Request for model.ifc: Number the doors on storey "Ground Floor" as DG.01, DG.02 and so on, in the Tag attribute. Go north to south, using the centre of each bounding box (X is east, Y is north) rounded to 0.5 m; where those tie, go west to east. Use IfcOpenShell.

First a look at what the model holds.

```python
import ifcopenshell
import ifcopenshell.util.element
import ifcopenshell.util.placement

model = ifcopenshell.open("model.ifc")
print(model.schema)
storey = next(s for s in model.by_type("IfcBuildingStorey") if s.Name == "Ground Floor")
doors = [e for e in ifcopenshell.util.element.get_decomposition(storey) if e.is_a("IfcDoor")]
for e in sorted(doors, key=lambda e: e.id()):
    origin = ifcopenshell.util.placement.get_local_placement(e.ObjectPlacement)[:3, 3]
    print(e.id(), e.Tag, e.Name, origin.round(2) + 0.0, sep=" | ")
```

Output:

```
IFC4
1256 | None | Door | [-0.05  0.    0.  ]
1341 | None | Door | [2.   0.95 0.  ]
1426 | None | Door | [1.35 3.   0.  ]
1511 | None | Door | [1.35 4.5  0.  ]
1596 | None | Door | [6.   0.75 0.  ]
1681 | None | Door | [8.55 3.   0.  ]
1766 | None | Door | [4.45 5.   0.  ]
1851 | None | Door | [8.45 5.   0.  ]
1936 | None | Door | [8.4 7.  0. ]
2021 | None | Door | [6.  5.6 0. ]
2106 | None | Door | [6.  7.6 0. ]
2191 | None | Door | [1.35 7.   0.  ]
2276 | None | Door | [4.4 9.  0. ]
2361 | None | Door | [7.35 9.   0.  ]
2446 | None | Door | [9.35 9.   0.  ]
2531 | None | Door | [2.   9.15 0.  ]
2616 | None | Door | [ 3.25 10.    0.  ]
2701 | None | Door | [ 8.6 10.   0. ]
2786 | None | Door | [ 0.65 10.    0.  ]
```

```python
import ifcopenshell
import ifcopenshell.geom
import ifcopenshell.util.element
import ifcopenshell.util.shape

model = ifcopenshell.open("model.ifc")
settings = ifcopenshell.geom.settings()
settings.set("use-world-coords", True)


def centre(element):
    shape = ifcopenshell.geom.create_shape(settings, element)
    return ifcopenshell.util.shape.get_bbox_centroid(shape.geometry)


storey = next(s for s in model.by_type("IfcBuildingStorey") if s.Name == "Ground Floor")
doors = [e for e in ifcopenshell.util.element.get_decomposition(storey) if e.is_a("IfcDoor")]

# Insertion points can sit at a corner or the storey origin, so sort by the geometry (in metres).
centres = {e: centre(e) for e in doors}
doors.sort(key=lambda e: (-round(centres[e][1] / 0.5), centres[e][0]))

for i, e in enumerate(doors, start=1):
    number = f"DG.{i:02d}"
    e.Tag = number
    print(e.id(), number)

model.write("model-out.ifc")
```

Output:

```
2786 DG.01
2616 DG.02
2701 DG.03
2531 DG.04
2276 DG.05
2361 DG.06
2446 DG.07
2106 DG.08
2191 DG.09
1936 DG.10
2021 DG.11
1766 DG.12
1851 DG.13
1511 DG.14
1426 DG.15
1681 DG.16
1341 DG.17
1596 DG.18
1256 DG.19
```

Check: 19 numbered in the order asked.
